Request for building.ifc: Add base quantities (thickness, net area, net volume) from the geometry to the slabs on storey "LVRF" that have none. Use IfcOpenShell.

First a look at what the model holds.

```python
import ifcopenshell
import ifcopenshell.util.element
import ifcopenshell.util.unit

model = ifcopenshell.open("building.ifc")
print(model.schema)
for unit_type in ("LENGTHUNIT", "AREAUNIT", "VOLUMEUNIT"):
    print(unit_type, ifcopenshell.util.unit.calculate_unit_scale(model, unit_type))
storey = next(s for s in model.by_type("IfcBuildingStorey") if s.Name == "LVRF")
slabs = [e for e in ifcopenshell.util.element.get_decomposition(storey) if e.is_a("IfcSlab")]
for e in sorted(slabs, key=lambda e: e.id()):
    print(e.id(), e.is_a(), e.Name, list(ifcopenshell.util.element.get_psets(e, qtos_only=True)), sep=" | ")
```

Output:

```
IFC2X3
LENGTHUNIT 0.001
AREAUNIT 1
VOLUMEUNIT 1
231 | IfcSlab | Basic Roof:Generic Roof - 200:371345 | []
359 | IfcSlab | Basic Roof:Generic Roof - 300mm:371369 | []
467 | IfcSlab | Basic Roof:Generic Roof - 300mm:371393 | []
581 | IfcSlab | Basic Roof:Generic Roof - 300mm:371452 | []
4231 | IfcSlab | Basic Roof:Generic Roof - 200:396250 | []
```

```python
import ifcopenshell
import ifcopenshell.api.pset
import ifcopenshell.geom
import ifcopenshell.util.element
import ifcopenshell.util.shape
import ifcopenshell.util.unit

model = ifcopenshell.open("building.ifc")
unit_scale = ifcopenshell.util.unit.calculate_unit_scale(model)
area_scale = ifcopenshell.util.unit.calculate_unit_scale(model, "AREAUNIT")
volume_scale = ifcopenshell.util.unit.calculate_unit_scale(model, "VOLUMEUNIT")
settings = ifcopenshell.geom.settings()

storey = next(s for s in model.by_type("IfcBuildingStorey") if s.Name == "LVRF")
slabs = [e for e in ifcopenshell.util.element.get_decomposition(storey) if e.is_a("IfcSlab")]

for e in sorted(slabs, key=lambda e: e.id()):
    if ifcopenshell.util.element.get_psets(e, qtos_only=True, should_inherit=False):
        continue
    # Geometry comes back in metres, in the element's own axes.
    shape = ifcopenshell.geom.create_shape(settings, e)
    values = {
        "Width": ifcopenshell.util.shape.get_z(shape.geometry) / unit_scale,
        "NetArea": ifcopenshell.util.shape.get_footprint_area(shape.geometry) / area_scale,
        "NetVolume": ifcopenshell.util.shape.get_volume(shape.geometry) / volume_scale,
    }
    qto = ifcopenshell.api.pset.add_qto(model, product=e, name="BaseQuantities")
    ifcopenshell.api.pset.edit_qto(model, qto=qto, properties=values)
    print(e.id(), {k: round(v, 3) for k, v in values.items()})

model.write("building_edited.ifc")
```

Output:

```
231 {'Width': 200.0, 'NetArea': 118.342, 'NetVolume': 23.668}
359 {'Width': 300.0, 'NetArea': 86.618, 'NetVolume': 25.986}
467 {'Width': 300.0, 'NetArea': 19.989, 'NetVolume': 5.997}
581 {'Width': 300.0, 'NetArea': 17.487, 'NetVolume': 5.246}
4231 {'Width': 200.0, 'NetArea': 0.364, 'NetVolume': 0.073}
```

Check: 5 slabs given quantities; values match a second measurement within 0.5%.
